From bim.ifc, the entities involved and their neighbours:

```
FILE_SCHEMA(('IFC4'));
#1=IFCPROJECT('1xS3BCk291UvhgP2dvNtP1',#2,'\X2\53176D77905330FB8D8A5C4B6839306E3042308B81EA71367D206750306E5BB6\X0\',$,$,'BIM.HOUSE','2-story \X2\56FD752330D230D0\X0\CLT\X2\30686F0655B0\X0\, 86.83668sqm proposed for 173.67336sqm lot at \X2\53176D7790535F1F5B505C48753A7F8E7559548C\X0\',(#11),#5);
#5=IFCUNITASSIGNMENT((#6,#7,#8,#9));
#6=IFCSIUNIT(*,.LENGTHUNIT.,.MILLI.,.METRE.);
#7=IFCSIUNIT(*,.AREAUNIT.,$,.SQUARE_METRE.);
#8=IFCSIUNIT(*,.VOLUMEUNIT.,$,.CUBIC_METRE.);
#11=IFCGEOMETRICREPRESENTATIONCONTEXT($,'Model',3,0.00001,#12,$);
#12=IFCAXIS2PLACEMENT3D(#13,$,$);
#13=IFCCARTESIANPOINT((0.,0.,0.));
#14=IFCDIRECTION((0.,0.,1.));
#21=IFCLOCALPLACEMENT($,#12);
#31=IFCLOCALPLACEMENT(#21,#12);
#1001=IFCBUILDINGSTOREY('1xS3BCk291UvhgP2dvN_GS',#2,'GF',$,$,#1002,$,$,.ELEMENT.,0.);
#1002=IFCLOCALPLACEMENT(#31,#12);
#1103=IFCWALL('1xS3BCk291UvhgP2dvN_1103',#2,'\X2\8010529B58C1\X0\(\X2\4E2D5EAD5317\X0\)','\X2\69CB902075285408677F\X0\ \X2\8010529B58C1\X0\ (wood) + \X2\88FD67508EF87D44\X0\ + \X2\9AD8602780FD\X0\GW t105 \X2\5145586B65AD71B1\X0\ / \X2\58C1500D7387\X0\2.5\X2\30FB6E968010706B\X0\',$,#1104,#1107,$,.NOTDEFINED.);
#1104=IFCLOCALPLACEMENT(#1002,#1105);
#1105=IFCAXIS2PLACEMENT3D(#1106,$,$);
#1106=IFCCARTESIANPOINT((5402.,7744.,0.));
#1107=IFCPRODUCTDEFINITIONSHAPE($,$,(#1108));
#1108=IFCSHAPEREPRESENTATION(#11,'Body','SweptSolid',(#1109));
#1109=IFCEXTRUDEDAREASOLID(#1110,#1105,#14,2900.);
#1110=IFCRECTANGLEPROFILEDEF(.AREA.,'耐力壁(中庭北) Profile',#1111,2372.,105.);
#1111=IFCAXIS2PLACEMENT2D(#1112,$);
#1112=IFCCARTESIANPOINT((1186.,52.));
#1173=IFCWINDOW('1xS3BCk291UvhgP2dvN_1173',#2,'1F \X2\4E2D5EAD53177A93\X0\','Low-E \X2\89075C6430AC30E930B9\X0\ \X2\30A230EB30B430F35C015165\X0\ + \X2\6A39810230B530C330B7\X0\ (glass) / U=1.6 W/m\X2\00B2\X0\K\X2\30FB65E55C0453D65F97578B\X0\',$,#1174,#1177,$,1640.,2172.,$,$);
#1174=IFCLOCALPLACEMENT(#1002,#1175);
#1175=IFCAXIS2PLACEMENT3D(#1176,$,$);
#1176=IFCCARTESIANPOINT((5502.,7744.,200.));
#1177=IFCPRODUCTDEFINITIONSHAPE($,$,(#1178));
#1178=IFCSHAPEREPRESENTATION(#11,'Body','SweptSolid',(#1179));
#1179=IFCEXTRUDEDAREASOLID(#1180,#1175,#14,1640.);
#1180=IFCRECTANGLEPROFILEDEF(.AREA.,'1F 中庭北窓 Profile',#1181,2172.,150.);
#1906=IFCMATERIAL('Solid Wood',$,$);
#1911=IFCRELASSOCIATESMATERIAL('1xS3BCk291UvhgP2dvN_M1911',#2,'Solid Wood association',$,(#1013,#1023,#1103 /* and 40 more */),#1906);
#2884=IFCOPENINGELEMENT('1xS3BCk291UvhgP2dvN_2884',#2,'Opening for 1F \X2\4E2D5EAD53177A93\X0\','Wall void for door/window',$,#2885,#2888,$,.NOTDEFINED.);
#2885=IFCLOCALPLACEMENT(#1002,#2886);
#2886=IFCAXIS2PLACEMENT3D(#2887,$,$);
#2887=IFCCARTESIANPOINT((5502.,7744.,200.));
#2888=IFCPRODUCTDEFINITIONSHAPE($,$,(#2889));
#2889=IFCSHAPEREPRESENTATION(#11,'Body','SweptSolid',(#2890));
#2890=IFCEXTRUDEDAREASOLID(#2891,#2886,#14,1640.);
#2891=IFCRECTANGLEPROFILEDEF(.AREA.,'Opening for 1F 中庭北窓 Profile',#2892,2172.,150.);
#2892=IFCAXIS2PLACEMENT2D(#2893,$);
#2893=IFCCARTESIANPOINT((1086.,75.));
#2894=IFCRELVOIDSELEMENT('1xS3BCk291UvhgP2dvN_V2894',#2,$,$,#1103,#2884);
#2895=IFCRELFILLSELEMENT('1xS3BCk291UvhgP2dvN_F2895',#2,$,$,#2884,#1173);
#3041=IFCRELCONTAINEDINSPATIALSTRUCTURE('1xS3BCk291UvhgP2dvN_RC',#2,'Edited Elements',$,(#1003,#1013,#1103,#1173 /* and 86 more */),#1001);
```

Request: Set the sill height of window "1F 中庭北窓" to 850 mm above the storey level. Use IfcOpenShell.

```python
import numpy as np
import ifcopenshell
import ifcopenshell.api.geometry
import ifcopenshell.geom
import ifcopenshell.util.element
import ifcopenshell.util.placement
import ifcopenshell.util.shape
import ifcopenshell.util.unit

model = ifcopenshell.open("bim.ifc")
unit_scale = ifcopenshell.util.unit.calculate_unit_scale(model)

window = model.by_id(1173)
opening = window.FillsVoids[0].RelatingOpeningElement
storey = ifcopenshell.util.element.get_container(window, ifc_class="IfcBuildingStorey")
level = ifcopenshell.util.placement.get_local_placement(storey.ObjectPlacement)[2, 3]

# The opening's origin need not be at the sill, so measure its lowest point.
shape = ifcopenshell.geom.create_shape(ifcopenshell.geom.settings(), opening)
bottom = ifcopenshell.util.shape.get_shape_bottom_elevation(shape, shape.geometry) / unit_scale
dz = level + 0.85 / unit_scale - bottom

shift = np.array([0.0, 0.0, dz])
# The window is not placed relative to its opening, so move both.
for product in (opening, window):
    matrix = ifcopenshell.util.placement.get_local_placement(product.ObjectPlacement)
    matrix[:3, 3] += shift
    ifcopenshell.api.geometry.edit_object_placement(model, product=product, matrix=matrix, is_si=False)

print(f"moved by {dz * unit_scale:+.3f} m")

model.write("bim_v2.ifc")
```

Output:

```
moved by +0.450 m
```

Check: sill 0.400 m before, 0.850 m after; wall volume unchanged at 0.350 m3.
